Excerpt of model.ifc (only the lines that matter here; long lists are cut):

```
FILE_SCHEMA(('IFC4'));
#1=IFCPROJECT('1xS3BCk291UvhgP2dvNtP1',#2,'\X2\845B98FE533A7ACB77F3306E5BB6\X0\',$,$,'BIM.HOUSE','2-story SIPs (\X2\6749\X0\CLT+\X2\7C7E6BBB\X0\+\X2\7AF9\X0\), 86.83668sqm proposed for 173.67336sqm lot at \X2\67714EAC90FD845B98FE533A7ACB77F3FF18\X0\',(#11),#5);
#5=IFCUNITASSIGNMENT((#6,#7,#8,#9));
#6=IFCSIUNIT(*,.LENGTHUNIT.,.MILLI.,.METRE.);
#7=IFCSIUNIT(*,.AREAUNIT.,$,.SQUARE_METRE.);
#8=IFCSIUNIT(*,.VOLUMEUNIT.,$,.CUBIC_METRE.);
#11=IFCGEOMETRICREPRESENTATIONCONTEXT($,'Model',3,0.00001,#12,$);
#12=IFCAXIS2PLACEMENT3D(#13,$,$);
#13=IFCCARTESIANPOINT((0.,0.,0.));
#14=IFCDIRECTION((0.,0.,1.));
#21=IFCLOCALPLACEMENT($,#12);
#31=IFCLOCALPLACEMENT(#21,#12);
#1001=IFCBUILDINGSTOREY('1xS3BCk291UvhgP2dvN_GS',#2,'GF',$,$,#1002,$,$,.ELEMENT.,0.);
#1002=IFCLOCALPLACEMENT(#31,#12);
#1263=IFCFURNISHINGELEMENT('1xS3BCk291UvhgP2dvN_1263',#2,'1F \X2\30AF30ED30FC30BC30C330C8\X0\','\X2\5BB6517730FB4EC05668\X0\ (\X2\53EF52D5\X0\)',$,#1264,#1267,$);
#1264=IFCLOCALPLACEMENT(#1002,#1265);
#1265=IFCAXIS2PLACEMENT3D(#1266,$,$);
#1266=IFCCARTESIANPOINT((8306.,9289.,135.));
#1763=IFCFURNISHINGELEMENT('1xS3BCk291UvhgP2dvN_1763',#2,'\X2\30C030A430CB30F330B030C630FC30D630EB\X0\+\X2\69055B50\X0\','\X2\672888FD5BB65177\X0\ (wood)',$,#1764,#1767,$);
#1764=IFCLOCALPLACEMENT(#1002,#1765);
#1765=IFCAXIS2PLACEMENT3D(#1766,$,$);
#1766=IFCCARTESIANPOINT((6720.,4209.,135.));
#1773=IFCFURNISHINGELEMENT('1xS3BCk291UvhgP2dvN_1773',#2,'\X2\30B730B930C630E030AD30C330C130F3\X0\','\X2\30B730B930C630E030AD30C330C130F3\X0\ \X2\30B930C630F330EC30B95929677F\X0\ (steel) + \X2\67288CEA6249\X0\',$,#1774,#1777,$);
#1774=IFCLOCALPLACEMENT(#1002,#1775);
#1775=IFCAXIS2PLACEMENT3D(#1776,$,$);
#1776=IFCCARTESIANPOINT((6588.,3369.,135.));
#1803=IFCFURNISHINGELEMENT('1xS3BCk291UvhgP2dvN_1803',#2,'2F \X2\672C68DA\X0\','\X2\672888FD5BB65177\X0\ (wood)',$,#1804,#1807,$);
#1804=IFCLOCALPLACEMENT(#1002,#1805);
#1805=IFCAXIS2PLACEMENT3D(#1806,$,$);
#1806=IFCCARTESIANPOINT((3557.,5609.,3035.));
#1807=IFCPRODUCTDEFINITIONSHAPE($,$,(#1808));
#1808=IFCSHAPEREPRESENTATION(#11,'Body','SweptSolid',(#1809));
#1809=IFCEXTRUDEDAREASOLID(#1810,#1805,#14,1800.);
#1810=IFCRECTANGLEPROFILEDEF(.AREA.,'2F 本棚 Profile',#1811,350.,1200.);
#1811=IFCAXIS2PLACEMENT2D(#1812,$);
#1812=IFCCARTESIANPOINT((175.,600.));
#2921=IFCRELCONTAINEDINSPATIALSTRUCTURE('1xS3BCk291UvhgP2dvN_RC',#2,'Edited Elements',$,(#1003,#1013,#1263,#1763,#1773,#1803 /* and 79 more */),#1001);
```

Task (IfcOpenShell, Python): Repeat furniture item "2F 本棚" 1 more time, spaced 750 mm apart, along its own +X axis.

```python
import ifcopenshell
import ifcopenshell.api.geometry
import ifcopenshell.api.root
import ifcopenshell.util.element
import ifcopenshell.util.placement
import ifcopenshell.util.unit

model = ifcopenshell.open("model.ifc")
unit_scale = ifcopenshell.util.unit.calculate_unit_scale(model)


def reuse_history(source, copy):
    """copy_class also copies each property set's owner history, people and application; keep the originals."""
    for rel in copy.IsDefinedBy:
        if rel.is_a("IfcRelDefinesByProperties") and (history := rel.RelatingPropertyDefinition.OwnerHistory):
            rel.RelatingPropertyDefinition.OwnerHistory = source.OwnerHistory
            ifcopenshell.util.element.remove_deep2(model, history)


source = model.by_guid("1xS3BCk291UvhgP2dvN_1803")
base = ifcopenshell.util.placement.get_local_placement(source.ObjectPlacement)
step = base[:3, 0] * 0.75 / unit_scale

for i in range(1, 2):
    copy = ifcopenshell.api.root.copy_class(model, product=source)
    copy.Representation = ifcopenshell.util.element.copy_deep(
        model, source.Representation, exclude=["IfcGeometricRepresentationContext", "IfcRepresentationMap"]
    )
    reuse_history(source, copy)
    matrix = base.copy()
    matrix[:3, 3] += i * step
    print("added at", matrix[:3, 3].round(3) + 0.0)
    ifcopenshell.api.geometry.edit_object_placement(model, product=copy, matrix=matrix, is_si=False)

model.write("model_v2.ifc")
```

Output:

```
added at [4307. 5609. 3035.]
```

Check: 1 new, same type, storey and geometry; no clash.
